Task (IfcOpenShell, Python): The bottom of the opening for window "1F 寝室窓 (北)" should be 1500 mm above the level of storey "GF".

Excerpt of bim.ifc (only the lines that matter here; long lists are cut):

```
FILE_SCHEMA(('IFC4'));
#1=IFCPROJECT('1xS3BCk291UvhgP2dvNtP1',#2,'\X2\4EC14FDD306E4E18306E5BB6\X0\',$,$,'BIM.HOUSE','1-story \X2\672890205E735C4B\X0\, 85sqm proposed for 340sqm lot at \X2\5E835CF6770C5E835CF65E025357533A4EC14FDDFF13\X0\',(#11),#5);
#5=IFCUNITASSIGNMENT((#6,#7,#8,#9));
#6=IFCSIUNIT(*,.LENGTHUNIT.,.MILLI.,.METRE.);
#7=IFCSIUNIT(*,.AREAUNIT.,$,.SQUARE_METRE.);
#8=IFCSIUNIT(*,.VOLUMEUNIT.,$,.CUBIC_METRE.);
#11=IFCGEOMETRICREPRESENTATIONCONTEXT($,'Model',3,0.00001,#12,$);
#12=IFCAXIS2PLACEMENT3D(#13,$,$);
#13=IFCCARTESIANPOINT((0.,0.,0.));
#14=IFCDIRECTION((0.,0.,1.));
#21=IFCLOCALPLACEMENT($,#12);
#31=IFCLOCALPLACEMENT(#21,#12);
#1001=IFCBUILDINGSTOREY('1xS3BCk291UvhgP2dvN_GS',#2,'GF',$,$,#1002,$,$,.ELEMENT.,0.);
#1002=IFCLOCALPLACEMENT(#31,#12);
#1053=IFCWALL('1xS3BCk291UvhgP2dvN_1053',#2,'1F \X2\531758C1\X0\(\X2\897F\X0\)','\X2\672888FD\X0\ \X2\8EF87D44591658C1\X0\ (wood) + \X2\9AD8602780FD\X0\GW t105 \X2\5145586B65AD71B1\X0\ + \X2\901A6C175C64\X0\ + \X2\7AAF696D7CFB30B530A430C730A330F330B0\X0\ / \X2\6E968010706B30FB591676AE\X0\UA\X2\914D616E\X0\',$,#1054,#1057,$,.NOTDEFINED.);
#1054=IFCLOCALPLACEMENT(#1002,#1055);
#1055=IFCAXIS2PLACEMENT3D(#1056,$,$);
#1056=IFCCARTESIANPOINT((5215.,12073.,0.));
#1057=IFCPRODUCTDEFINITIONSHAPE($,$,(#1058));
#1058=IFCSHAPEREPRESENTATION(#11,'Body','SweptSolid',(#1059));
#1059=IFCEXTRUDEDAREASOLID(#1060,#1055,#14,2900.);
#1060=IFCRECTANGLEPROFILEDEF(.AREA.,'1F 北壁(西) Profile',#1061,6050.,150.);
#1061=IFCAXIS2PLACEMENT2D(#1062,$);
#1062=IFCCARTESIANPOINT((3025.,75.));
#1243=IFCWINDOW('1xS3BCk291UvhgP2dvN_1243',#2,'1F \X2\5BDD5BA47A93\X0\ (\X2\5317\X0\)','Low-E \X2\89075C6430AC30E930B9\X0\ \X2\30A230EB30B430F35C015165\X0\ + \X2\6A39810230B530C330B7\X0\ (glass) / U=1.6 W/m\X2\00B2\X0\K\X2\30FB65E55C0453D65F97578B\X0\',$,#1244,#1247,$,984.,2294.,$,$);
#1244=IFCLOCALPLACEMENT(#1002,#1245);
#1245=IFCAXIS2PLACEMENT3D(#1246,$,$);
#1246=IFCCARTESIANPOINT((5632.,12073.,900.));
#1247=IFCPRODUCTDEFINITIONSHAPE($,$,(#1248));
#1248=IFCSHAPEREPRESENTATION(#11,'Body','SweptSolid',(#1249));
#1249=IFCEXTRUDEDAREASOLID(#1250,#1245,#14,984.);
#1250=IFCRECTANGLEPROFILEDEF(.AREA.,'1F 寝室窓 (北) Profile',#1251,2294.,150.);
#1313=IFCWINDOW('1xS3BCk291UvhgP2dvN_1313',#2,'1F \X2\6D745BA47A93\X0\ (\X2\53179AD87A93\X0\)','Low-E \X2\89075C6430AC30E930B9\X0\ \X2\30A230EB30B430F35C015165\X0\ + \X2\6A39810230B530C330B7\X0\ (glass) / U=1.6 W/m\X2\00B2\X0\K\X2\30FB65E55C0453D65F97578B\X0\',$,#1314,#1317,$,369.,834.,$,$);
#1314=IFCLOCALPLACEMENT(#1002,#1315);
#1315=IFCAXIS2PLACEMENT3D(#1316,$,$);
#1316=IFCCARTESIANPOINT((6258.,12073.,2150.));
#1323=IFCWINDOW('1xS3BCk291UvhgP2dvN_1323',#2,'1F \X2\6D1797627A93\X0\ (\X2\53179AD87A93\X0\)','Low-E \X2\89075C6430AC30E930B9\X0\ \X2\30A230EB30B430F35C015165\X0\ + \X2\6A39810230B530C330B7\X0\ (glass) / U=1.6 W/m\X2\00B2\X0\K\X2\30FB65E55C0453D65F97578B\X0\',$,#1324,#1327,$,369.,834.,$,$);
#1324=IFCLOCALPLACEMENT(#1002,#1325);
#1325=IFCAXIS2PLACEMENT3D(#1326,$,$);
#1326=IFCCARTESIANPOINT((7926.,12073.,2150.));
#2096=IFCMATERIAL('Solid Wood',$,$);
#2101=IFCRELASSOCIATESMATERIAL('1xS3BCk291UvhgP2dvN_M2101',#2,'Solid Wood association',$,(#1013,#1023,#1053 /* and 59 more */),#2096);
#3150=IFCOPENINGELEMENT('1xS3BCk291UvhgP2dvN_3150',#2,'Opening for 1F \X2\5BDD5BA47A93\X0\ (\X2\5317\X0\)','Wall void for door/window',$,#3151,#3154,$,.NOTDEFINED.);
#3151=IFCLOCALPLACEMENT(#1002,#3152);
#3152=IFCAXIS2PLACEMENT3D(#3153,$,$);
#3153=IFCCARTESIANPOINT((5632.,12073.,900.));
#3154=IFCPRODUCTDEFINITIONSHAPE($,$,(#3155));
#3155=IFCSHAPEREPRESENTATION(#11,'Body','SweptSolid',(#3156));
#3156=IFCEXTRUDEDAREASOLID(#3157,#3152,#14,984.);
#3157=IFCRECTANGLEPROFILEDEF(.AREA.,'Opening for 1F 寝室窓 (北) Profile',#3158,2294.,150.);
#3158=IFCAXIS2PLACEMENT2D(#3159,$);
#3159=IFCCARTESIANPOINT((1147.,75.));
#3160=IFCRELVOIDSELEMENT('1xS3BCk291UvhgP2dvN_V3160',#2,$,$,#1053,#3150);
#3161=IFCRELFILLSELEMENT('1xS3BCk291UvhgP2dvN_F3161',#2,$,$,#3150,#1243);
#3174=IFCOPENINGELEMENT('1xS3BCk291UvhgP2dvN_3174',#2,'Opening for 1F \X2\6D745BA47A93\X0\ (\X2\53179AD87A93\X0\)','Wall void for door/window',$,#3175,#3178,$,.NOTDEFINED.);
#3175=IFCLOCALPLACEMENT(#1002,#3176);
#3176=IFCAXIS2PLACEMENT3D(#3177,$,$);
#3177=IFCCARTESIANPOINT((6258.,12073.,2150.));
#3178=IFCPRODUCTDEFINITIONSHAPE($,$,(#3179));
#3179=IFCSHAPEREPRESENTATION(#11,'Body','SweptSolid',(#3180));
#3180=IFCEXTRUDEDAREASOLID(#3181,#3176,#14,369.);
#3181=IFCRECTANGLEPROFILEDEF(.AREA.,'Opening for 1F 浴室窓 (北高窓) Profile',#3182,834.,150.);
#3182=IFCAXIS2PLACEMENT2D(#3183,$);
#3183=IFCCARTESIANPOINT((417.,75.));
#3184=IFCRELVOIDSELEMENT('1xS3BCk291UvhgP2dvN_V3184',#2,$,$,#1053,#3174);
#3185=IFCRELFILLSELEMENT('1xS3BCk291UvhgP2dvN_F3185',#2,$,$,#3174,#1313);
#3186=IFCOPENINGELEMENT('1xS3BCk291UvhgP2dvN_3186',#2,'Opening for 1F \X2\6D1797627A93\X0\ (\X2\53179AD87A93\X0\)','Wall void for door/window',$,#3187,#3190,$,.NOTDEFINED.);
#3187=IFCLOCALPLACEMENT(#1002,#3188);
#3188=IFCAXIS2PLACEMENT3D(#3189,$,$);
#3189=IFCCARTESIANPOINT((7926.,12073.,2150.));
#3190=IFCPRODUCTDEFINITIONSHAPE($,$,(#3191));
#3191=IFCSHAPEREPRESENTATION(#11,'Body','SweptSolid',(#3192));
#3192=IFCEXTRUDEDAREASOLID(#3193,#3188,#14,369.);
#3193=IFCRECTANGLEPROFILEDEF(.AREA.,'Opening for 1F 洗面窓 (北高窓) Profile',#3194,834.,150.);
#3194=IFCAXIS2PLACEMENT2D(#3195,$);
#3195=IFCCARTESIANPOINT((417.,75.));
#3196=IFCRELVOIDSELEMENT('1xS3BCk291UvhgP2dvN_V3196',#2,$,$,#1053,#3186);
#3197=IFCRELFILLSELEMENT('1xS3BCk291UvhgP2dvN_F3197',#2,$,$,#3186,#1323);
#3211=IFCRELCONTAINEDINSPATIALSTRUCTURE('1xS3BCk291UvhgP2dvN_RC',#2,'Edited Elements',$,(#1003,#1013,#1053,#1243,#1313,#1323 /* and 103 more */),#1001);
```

```python
import numpy as np
import ifcopenshell
import ifcopenshell.api.geometry
import ifcopenshell.geom
import ifcopenshell.util.element
import ifcopenshell.util.placement
import ifcopenshell.util.shape
import ifcopenshell.util.unit

model = ifcopenshell.open("bim.ifc")
unit_scale = ifcopenshell.util.unit.calculate_unit_scale(model)

window = model.by_id(1243)
opening = window.FillsVoids[0].RelatingOpeningElement
storey = ifcopenshell.util.element.get_container(window, ifc_class="IfcBuildingStorey")
level = ifcopenshell.util.placement.get_local_placement(storey.ObjectPlacement)[2, 3]

# The opening's origin need not be at the sill, so measure its lowest point.
shape = ifcopenshell.geom.create_shape(ifcopenshell.geom.settings(), opening)
bottom = ifcopenshell.util.shape.get_shape_bottom_elevation(shape, shape.geometry) / unit_scale
dz = level + 1.5 / unit_scale - bottom

shift = np.array([0.0, 0.0, dz])
# The window is not placed relative to its opening, so move both.
for product in (opening, window):
    matrix = ifcopenshell.util.placement.get_local_placement(product.ObjectPlacement)
    matrix[:3, 3] += shift
    ifcopenshell.api.geometry.edit_object_placement(model, product=product, matrix=matrix, is_si=False)

print(f"moved by {dz * unit_scale:+.3f} m")

model.write("bim_v2.ifc")
```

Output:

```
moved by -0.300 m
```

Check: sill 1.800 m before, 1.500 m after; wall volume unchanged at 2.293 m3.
